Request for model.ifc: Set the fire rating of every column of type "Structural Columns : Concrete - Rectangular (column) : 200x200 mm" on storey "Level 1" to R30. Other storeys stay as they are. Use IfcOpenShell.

First a look at what the model holds.

```python
import ifcopenshell
import ifcopenshell.util.element

model = ifcopenshell.open("model.ifc")
print(model.schema)
storey = next(s for s in model.by_type("IfcBuildingStorey") if s.Name == "Level 1")
columns = [e for e in ifcopenshell.util.element.get_decomposition(storey) if e.is_a("IfcColumn")]
seen = {}
for e in columns:
    element_type = ifcopenshell.util.element.get_type(e)
    key = (element_type.Name if element_type != e and element_type else None, ifcopenshell.util.element.get_pset(e, "Pset_ColumnCommon", "FireRating"))
    seen[key] = seen.get(key, 0) + 1
for (name, value), count in sorted(seen.items(), key=str):
    print(count, "x", name, "|", value)
```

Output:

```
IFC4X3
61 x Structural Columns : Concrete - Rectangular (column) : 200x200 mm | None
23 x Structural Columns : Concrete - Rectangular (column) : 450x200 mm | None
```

```python
import ifcopenshell
import ifcopenshell.api.pset
import ifcopenshell.util.element

model = ifcopenshell.open("model.ifc")

storey = next(s for s in model.by_type("IfcBuildingStorey") if s.Name == "Level 1")
columns = [e for e in ifcopenshell.util.element.get_decomposition(storey) if e.is_a("IfcColumn")]

count = 0
for e in columns:
    element_type = ifcopenshell.util.element.get_type(e)
    if element_type in (None, e) or element_type.Name != "Structural Columns : Concrete - Rectangular (column) : 200x200 mm":
        continue
    # add_pset returns the element's existing set when there is one.
    pset = ifcopenshell.api.pset.add_pset(model, product=e, name="Pset_ColumnCommon")
    ifcopenshell.api.pset.edit_pset(model, pset=pset, properties={"FireRating": "R30"})
    count += 1

print(count, "columns updated")

model.write("model_v2.ifc")
```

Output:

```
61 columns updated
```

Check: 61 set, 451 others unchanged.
